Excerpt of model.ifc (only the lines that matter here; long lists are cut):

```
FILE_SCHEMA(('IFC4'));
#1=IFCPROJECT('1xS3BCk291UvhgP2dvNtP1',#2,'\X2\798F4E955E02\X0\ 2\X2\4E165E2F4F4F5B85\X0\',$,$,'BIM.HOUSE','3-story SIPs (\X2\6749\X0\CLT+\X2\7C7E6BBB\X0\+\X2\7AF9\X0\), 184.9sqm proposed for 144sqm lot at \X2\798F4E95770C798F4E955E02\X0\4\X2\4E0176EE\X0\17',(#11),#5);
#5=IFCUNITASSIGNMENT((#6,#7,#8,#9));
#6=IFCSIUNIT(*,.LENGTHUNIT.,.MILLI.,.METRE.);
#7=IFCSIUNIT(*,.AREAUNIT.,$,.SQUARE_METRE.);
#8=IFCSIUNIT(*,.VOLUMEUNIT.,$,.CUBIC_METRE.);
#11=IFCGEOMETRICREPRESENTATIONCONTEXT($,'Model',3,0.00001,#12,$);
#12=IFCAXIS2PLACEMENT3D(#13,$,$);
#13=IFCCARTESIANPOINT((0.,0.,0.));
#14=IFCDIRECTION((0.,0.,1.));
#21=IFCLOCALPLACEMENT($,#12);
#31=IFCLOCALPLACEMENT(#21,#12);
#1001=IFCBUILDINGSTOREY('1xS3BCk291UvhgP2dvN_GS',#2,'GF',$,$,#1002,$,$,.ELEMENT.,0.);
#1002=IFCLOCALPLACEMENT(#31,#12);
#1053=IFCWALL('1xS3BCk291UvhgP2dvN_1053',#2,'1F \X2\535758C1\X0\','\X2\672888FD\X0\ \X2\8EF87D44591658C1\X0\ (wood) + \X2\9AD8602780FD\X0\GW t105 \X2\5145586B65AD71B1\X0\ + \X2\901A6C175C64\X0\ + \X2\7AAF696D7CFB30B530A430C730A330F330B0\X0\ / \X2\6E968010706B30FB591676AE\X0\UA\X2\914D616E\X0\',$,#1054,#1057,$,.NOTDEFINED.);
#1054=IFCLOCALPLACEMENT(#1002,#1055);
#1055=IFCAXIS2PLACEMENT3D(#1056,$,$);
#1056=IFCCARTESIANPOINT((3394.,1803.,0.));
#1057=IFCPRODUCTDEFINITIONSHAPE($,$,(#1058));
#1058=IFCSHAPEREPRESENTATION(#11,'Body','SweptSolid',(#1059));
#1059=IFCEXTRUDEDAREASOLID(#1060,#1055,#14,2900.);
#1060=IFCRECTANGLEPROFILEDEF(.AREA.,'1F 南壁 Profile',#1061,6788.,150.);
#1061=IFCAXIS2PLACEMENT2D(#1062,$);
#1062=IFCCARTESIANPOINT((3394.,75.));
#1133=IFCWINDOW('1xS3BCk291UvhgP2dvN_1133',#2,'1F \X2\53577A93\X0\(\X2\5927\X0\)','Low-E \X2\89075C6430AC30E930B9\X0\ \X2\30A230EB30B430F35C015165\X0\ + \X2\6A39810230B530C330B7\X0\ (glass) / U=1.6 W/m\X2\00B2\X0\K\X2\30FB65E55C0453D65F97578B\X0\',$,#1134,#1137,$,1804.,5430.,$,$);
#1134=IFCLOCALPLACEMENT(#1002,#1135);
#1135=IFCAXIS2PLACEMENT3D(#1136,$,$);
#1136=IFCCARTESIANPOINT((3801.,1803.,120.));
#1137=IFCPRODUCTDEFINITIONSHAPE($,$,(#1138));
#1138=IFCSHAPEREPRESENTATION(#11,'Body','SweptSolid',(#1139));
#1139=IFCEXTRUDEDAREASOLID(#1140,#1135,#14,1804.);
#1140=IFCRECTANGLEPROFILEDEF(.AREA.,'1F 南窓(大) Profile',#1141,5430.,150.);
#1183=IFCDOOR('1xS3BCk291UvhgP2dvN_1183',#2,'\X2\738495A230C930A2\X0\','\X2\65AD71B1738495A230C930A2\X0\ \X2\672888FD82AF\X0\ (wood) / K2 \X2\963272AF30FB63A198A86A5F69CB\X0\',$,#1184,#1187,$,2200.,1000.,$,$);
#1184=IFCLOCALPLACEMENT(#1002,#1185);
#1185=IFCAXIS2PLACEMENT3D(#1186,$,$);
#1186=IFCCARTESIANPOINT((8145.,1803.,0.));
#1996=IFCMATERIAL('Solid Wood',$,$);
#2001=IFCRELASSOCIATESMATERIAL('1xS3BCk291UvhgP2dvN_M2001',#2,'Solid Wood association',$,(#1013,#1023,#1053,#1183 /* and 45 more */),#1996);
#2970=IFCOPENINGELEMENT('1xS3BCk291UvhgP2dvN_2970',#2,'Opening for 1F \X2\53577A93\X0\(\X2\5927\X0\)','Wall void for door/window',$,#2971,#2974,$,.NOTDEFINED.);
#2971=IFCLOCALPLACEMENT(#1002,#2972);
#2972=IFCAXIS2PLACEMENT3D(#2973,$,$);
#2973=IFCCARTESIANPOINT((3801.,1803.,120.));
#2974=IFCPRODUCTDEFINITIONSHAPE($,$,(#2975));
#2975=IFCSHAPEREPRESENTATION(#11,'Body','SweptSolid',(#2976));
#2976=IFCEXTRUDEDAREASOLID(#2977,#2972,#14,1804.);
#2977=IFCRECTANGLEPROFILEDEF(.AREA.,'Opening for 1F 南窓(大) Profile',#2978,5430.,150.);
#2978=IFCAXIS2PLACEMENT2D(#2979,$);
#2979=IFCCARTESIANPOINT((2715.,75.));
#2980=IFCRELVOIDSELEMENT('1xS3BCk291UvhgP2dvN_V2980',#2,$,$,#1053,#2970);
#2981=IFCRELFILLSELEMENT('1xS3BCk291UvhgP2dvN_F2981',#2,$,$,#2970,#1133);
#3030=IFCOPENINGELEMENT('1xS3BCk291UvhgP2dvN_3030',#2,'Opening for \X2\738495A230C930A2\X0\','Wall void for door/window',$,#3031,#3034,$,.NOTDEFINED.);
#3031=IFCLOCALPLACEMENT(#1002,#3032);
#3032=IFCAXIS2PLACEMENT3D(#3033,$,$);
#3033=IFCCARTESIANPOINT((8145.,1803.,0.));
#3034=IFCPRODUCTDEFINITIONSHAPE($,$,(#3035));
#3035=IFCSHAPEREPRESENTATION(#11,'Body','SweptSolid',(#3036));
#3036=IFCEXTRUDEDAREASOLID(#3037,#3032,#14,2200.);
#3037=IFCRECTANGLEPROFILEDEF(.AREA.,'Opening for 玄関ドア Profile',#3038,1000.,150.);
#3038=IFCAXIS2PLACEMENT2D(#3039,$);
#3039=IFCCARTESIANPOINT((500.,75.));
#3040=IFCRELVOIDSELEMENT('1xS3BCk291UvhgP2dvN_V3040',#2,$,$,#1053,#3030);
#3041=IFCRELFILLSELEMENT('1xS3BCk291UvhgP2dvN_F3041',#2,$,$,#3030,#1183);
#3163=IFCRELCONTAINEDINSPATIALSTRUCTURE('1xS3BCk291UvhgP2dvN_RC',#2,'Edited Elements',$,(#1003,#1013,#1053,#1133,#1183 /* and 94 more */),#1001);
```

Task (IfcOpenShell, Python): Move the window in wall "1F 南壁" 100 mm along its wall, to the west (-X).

```python
import ifcopenshell
import ifcopenshell.api.geometry
import ifcopenshell.util.placement

model = ifcopenshell.open("model.ifc")

window = model.by_id(1133)
opening = window.FillsVoids[0].RelatingOpeningElement
wall = opening.VoidsElements[0].RelatingBuildingElement

wall_matrix = ifcopenshell.util.placement.get_local_placement(wall.ObjectPlacement)
shift = wall_matrix[:3, 0] * -100.0
before = ifcopenshell.util.placement.get_local_placement(window.ObjectPlacement)[:3, 3].copy()

# The window is not placed relative to its opening, so move both.
for product in (opening, window):
    matrix = ifcopenshell.util.placement.get_local_placement(product.ObjectPlacement)
    matrix[:3, 3] += shift
    ifcopenshell.api.geometry.edit_object_placement(model, product=product, matrix=matrix, is_si=False)

after = ifcopenshell.util.placement.get_local_placement(window.ObjectPlacement)[:3, 3]
print("window moved by", (after - before).round(3) + 0.0)

model.write("model_updated.ifc")
```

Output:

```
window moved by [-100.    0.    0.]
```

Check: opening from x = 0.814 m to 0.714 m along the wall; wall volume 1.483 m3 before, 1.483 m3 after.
